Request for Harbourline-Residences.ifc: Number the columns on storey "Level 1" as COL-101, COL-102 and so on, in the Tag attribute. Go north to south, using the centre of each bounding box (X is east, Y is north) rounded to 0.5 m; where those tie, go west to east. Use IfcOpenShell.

First a look at what the model holds.

```python
import ifcopenshell
import ifcopenshell.util.element
import ifcopenshell.util.placement

model = ifcopenshell.open("Harbourline-Residences.ifc")
print(model.schema)
storey = next(s for s in model.by_type("IfcBuildingStorey") if s.Name == "Level 1")
columns = [e for e in ifcopenshell.util.element.get_decomposition(storey) if e.is_a("IfcColumn")]
for e in sorted(columns, key=lambda e: e.id()):
    origin = ifcopenshell.util.placement.get_local_placement(e.ObjectPlacement)[:3, 3]
    print(e.id(), e.Tag, e.Name, origin.round(2) + 0.0, sep=" | ")
```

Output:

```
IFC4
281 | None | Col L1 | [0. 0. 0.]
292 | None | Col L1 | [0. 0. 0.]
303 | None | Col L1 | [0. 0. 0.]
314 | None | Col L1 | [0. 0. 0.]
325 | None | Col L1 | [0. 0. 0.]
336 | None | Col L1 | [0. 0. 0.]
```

```python
import ifcopenshell
import ifcopenshell.geom
import ifcopenshell.util.element
import ifcopenshell.util.shape

model = ifcopenshell.open("Harbourline-Residences.ifc")
settings = ifcopenshell.geom.settings()
settings.set("use-world-coords", True)


def centre(element):
    shape = ifcopenshell.geom.create_shape(settings, element)
    return ifcopenshell.util.shape.get_bbox_centroid(shape.geometry)


storey = next(s for s in model.by_type("IfcBuildingStorey") if s.Name == "Level 1")
columns = [e for e in ifcopenshell.util.element.get_decomposition(storey) if e.is_a("IfcColumn")]

# Insertion points can sit at a corner or the storey origin, so sort by the geometry (in metres).
centres = {e: centre(e) for e in columns}
columns.sort(key=lambda e: (-round(centres[e][1] / 0.5), centres[e][0]))

for i, e in enumerate(columns, start=1):
    number = f"COL-1{i:02d}"
    e.Tag = number
    print(e.id(), number)

model.write("Harbourline-Residences_rev.ifc")
```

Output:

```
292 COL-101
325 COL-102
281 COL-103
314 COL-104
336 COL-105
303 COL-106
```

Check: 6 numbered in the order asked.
